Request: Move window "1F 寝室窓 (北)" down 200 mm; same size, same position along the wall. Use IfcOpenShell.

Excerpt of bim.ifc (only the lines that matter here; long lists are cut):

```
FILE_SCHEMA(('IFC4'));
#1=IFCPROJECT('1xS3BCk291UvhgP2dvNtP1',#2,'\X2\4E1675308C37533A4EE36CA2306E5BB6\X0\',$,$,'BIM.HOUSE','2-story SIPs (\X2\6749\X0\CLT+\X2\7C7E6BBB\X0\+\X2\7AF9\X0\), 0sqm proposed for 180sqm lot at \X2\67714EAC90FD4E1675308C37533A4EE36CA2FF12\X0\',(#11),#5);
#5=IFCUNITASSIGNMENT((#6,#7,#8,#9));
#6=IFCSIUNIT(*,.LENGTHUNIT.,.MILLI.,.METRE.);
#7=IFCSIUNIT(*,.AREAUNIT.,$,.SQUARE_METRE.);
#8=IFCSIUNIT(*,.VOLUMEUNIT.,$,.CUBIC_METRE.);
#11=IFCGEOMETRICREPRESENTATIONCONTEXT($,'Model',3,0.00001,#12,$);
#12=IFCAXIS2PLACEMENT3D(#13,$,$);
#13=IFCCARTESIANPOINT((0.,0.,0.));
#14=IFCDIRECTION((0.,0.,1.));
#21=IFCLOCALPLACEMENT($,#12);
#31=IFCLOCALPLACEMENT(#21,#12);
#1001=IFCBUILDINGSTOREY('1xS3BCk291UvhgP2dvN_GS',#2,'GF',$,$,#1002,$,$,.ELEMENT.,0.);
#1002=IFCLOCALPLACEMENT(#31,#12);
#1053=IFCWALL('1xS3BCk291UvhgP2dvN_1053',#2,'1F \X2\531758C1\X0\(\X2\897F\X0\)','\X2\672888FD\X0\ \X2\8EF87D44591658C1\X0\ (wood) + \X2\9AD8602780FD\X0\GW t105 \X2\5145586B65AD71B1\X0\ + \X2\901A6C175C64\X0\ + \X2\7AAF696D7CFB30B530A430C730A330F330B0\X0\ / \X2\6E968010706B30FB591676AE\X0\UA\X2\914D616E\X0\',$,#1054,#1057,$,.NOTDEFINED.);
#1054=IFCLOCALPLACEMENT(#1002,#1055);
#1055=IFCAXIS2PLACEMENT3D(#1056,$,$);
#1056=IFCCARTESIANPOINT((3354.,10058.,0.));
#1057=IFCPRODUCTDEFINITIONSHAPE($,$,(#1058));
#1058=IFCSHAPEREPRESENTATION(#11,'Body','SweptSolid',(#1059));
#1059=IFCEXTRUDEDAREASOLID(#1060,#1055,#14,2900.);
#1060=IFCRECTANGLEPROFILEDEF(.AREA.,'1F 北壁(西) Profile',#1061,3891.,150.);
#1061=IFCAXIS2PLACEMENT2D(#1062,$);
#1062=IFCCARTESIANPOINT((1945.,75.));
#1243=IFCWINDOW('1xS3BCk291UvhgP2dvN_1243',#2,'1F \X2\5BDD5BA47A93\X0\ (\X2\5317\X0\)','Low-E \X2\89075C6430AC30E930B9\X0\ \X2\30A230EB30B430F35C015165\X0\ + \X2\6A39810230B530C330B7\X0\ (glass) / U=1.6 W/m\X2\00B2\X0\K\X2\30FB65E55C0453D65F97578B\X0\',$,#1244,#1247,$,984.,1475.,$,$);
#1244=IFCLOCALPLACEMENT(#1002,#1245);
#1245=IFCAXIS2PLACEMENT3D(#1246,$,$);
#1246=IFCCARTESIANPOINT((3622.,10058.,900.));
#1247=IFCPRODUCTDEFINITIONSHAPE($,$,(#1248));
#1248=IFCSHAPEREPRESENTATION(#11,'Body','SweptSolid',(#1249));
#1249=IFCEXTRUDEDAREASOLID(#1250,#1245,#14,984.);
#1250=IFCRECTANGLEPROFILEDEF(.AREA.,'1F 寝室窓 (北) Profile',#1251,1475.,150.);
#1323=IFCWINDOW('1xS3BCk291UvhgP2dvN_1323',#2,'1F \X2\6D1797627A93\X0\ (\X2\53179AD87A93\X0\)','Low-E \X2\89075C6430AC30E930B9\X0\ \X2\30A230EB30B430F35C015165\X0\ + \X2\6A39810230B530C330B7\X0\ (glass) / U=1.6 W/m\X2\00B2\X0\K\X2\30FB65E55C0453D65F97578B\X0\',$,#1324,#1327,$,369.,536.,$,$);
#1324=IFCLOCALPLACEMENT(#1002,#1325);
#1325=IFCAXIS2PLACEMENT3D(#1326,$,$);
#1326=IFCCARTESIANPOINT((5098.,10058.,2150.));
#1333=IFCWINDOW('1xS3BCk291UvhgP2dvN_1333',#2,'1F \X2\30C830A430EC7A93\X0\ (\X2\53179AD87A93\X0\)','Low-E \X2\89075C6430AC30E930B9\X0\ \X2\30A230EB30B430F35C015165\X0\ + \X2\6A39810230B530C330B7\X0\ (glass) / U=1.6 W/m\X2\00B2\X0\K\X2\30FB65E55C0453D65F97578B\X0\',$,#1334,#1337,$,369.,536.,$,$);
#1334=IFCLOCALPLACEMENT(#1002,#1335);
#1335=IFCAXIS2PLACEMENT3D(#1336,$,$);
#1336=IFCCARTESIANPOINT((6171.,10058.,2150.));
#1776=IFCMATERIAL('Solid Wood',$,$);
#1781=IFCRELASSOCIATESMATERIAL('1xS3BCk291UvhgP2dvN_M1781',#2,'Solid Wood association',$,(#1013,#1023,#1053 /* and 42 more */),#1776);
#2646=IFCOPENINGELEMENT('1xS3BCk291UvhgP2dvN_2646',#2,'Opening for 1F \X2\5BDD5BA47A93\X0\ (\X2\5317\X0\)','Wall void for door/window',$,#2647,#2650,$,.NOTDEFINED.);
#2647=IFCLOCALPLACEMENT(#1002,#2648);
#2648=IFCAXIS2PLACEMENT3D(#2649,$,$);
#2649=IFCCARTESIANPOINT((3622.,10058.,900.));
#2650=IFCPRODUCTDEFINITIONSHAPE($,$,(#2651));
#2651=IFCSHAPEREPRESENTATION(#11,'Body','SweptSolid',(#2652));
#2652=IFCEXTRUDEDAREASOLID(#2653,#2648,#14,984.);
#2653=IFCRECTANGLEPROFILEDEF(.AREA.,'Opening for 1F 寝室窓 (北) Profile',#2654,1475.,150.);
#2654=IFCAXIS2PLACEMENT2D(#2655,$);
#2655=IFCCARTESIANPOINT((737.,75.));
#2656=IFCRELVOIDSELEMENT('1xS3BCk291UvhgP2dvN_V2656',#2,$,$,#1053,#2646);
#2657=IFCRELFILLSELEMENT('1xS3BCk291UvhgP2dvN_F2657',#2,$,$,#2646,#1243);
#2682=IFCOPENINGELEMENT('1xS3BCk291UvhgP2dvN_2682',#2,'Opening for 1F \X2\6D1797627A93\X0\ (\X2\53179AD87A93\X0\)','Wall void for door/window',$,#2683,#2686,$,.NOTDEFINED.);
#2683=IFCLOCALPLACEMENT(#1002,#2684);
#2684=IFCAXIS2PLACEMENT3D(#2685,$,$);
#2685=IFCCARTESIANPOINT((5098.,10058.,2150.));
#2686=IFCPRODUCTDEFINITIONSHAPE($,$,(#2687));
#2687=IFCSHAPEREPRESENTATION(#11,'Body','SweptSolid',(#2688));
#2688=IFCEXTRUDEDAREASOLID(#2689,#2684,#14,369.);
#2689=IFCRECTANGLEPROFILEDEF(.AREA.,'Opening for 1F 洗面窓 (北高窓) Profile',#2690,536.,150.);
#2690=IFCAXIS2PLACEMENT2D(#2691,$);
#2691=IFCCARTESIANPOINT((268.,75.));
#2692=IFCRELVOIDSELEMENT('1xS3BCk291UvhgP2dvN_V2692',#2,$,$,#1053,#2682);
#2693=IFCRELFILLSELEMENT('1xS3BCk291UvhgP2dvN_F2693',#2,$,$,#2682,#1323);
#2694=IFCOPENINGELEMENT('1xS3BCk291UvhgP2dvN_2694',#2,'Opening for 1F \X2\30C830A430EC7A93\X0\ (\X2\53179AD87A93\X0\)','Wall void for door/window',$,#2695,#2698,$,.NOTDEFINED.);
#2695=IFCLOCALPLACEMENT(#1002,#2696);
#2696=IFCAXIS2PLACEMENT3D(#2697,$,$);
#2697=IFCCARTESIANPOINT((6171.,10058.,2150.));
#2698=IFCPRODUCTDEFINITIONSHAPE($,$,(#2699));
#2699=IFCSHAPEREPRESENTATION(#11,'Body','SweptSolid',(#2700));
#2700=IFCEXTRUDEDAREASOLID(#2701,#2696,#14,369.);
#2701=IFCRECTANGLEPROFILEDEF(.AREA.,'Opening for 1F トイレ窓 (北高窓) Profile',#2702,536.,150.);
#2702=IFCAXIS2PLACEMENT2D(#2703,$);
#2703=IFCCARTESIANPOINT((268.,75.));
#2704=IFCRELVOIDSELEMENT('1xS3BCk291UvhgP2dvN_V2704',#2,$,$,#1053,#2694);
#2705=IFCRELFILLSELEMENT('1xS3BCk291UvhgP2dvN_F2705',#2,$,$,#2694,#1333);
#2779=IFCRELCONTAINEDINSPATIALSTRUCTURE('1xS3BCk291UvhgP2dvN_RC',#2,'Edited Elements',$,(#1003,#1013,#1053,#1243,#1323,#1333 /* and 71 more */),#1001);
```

```python
import numpy as np
import ifcopenshell
import ifcopenshell.api.geometry
import ifcopenshell.util.placement
import ifcopenshell.util.unit

model = ifcopenshell.open("bim.ifc")
unit_scale = ifcopenshell.util.unit.calculate_unit_scale(model)

window = model.by_id(1243)
opening = window.FillsVoids[0].RelatingOpeningElement
dz = -200.0

shift = np.array([0.0, 0.0, dz])
# The window is not placed relative to its opening, so move both.
for product in (opening, window):
    matrix = ifcopenshell.util.placement.get_local_placement(product.ObjectPlacement)
    matrix[:3, 3] += shift
    ifcopenshell.api.geometry.edit_object_placement(model, product=product, matrix=matrix, is_si=False)

print(f"moved by {dz * unit_scale:+.3f} m")

model.write("bim_updated.ifc")
```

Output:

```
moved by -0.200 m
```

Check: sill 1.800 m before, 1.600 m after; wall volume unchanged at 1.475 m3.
